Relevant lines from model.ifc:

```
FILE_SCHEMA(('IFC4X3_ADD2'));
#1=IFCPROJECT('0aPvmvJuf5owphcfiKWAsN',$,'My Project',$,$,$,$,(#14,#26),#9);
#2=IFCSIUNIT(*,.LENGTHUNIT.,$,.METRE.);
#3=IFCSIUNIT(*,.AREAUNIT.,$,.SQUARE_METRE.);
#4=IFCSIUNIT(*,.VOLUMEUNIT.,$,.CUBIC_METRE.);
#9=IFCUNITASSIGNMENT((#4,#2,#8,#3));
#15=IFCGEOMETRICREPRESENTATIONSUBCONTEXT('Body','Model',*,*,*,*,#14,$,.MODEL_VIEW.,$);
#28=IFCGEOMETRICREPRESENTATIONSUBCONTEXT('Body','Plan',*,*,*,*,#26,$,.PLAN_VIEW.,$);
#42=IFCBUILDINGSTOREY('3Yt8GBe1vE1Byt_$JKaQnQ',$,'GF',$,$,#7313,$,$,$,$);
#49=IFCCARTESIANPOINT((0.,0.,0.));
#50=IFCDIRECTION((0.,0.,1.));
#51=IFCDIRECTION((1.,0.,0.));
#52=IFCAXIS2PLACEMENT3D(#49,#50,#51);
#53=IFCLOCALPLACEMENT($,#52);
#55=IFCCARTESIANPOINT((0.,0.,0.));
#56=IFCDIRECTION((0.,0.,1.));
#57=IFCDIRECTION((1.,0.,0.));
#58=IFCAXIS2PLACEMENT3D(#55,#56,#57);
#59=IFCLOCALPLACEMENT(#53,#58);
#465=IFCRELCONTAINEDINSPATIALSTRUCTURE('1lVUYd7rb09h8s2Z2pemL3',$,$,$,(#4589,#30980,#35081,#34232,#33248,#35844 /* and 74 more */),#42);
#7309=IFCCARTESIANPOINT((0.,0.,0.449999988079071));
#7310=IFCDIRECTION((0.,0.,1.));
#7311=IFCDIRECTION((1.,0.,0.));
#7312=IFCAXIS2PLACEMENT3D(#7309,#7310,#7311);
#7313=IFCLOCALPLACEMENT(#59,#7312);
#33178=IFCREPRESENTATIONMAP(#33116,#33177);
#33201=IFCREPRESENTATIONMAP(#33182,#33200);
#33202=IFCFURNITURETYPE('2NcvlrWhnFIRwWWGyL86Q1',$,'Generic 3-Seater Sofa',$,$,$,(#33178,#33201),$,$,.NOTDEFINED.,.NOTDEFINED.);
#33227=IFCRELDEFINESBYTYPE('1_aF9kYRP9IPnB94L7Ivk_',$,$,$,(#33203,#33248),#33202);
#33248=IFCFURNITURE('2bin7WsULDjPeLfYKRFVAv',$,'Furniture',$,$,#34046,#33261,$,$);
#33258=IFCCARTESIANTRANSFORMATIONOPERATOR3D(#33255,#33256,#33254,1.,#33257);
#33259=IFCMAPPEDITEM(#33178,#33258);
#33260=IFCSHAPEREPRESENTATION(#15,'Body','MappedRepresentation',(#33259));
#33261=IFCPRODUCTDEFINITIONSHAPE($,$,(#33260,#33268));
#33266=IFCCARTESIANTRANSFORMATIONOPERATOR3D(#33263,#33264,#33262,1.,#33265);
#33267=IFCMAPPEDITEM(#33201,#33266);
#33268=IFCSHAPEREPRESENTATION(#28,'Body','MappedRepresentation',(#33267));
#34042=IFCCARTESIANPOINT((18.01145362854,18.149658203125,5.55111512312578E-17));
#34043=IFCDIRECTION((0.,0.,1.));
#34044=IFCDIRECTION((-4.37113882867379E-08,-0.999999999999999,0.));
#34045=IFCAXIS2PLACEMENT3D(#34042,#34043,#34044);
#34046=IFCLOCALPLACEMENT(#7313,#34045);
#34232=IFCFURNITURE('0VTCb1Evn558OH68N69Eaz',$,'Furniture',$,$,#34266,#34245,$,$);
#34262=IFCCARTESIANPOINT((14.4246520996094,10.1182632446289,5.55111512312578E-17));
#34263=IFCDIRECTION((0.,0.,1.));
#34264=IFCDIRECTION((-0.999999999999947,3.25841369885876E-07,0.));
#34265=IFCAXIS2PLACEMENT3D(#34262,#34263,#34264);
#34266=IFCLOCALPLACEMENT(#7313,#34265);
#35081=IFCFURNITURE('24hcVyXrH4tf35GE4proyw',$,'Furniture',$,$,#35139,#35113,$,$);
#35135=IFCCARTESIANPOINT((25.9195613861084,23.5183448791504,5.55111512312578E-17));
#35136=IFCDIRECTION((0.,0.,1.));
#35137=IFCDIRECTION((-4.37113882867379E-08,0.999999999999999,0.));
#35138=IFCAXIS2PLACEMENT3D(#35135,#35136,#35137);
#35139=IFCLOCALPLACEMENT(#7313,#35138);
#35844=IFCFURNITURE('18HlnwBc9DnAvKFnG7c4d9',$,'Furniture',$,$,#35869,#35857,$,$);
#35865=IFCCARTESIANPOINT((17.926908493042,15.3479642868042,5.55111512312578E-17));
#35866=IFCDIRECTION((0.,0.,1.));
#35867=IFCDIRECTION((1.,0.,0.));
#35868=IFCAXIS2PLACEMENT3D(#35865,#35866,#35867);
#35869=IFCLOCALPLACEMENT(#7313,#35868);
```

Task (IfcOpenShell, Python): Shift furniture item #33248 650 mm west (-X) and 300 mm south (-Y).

```python
import ifcopenshell
import ifcopenshell.api.geometry
import ifcopenshell.util.placement

model = ifcopenshell.open("model.ifc")

item = model.by_id(33248)
matrix = ifcopenshell.util.placement.get_local_placement(item.ObjectPlacement)
matrix[0, 3] -= 0.65
matrix[1, 3] -= 0.3
ifcopenshell.api.geometry.edit_object_placement(model, product=item, matrix=matrix, is_si=False)

print(ifcopenshell.util.placement.get_local_placement(item.ObjectPlacement).round(3) + 0.0)

model.write("model_edited.ifc")
```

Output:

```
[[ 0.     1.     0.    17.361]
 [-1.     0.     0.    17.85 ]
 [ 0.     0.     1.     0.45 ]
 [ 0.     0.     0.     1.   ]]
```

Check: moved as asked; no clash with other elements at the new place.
